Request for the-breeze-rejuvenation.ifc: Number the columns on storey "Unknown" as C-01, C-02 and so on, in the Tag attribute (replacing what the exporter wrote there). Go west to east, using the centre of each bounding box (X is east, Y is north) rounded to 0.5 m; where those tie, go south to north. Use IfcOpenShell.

First a look at what the model holds.

```python
import ifcopenshell
import ifcopenshell.util.element
import ifcopenshell.util.placement

model = ifcopenshell.open("the-breeze-rejuvenation.ifc")
print(model.schema)
storey = next(s for s in model.by_type("IfcBuildingStorey") if s.Name == "Unknown")
columns = [e for e in ifcopenshell.util.element.get_decomposition(storey) if e.is_a("IfcColumn")]
for e in sorted(columns, key=lambda e: e.id()):
    origin = ifcopenshell.util.placement.get_local_placement(e.ObjectPlacement)[:3, 3]
    print(e.id(), e.Tag, e.Name, origin.round(2) + 0.0, sep=" | ")
```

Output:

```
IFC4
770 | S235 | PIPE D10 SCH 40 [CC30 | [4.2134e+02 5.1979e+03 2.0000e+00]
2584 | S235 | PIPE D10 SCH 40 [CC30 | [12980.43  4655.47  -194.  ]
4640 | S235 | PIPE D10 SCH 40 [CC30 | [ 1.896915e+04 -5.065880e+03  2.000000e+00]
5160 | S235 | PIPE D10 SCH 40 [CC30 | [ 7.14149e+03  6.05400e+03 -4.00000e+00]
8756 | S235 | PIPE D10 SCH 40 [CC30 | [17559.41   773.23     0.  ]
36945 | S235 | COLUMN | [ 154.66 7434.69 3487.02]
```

```python
import ifcopenshell
import ifcopenshell.geom
import ifcopenshell.util.element
import ifcopenshell.util.shape

model = ifcopenshell.open("the-breeze-rejuvenation.ifc")
settings = ifcopenshell.geom.settings()
settings.set("use-world-coords", True)


def centre(element):
    shape = ifcopenshell.geom.create_shape(settings, element)
    return ifcopenshell.util.shape.get_bbox_centroid(shape.geometry)


storey = next(s for s in model.by_type("IfcBuildingStorey") if s.Name == "Unknown")
columns = [e for e in ifcopenshell.util.element.get_decomposition(storey) if e.is_a("IfcColumn")]

# Insertion points can sit at a corner or the storey origin, so sort by the geometry (in metres).
centres = {e: centre(e) for e in columns}
columns.sort(key=lambda e: (round(centres[e][0] / 0.5), centres[e][1]))

for i, e in enumerate(columns, start=1):
    number = f"C-{i:02d}"
    e.Tag = number
    print(e.id(), number)

model.write("the-breeze-rejuvenation_rev.ifc")
```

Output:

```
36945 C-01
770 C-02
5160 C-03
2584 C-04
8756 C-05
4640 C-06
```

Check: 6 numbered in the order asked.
